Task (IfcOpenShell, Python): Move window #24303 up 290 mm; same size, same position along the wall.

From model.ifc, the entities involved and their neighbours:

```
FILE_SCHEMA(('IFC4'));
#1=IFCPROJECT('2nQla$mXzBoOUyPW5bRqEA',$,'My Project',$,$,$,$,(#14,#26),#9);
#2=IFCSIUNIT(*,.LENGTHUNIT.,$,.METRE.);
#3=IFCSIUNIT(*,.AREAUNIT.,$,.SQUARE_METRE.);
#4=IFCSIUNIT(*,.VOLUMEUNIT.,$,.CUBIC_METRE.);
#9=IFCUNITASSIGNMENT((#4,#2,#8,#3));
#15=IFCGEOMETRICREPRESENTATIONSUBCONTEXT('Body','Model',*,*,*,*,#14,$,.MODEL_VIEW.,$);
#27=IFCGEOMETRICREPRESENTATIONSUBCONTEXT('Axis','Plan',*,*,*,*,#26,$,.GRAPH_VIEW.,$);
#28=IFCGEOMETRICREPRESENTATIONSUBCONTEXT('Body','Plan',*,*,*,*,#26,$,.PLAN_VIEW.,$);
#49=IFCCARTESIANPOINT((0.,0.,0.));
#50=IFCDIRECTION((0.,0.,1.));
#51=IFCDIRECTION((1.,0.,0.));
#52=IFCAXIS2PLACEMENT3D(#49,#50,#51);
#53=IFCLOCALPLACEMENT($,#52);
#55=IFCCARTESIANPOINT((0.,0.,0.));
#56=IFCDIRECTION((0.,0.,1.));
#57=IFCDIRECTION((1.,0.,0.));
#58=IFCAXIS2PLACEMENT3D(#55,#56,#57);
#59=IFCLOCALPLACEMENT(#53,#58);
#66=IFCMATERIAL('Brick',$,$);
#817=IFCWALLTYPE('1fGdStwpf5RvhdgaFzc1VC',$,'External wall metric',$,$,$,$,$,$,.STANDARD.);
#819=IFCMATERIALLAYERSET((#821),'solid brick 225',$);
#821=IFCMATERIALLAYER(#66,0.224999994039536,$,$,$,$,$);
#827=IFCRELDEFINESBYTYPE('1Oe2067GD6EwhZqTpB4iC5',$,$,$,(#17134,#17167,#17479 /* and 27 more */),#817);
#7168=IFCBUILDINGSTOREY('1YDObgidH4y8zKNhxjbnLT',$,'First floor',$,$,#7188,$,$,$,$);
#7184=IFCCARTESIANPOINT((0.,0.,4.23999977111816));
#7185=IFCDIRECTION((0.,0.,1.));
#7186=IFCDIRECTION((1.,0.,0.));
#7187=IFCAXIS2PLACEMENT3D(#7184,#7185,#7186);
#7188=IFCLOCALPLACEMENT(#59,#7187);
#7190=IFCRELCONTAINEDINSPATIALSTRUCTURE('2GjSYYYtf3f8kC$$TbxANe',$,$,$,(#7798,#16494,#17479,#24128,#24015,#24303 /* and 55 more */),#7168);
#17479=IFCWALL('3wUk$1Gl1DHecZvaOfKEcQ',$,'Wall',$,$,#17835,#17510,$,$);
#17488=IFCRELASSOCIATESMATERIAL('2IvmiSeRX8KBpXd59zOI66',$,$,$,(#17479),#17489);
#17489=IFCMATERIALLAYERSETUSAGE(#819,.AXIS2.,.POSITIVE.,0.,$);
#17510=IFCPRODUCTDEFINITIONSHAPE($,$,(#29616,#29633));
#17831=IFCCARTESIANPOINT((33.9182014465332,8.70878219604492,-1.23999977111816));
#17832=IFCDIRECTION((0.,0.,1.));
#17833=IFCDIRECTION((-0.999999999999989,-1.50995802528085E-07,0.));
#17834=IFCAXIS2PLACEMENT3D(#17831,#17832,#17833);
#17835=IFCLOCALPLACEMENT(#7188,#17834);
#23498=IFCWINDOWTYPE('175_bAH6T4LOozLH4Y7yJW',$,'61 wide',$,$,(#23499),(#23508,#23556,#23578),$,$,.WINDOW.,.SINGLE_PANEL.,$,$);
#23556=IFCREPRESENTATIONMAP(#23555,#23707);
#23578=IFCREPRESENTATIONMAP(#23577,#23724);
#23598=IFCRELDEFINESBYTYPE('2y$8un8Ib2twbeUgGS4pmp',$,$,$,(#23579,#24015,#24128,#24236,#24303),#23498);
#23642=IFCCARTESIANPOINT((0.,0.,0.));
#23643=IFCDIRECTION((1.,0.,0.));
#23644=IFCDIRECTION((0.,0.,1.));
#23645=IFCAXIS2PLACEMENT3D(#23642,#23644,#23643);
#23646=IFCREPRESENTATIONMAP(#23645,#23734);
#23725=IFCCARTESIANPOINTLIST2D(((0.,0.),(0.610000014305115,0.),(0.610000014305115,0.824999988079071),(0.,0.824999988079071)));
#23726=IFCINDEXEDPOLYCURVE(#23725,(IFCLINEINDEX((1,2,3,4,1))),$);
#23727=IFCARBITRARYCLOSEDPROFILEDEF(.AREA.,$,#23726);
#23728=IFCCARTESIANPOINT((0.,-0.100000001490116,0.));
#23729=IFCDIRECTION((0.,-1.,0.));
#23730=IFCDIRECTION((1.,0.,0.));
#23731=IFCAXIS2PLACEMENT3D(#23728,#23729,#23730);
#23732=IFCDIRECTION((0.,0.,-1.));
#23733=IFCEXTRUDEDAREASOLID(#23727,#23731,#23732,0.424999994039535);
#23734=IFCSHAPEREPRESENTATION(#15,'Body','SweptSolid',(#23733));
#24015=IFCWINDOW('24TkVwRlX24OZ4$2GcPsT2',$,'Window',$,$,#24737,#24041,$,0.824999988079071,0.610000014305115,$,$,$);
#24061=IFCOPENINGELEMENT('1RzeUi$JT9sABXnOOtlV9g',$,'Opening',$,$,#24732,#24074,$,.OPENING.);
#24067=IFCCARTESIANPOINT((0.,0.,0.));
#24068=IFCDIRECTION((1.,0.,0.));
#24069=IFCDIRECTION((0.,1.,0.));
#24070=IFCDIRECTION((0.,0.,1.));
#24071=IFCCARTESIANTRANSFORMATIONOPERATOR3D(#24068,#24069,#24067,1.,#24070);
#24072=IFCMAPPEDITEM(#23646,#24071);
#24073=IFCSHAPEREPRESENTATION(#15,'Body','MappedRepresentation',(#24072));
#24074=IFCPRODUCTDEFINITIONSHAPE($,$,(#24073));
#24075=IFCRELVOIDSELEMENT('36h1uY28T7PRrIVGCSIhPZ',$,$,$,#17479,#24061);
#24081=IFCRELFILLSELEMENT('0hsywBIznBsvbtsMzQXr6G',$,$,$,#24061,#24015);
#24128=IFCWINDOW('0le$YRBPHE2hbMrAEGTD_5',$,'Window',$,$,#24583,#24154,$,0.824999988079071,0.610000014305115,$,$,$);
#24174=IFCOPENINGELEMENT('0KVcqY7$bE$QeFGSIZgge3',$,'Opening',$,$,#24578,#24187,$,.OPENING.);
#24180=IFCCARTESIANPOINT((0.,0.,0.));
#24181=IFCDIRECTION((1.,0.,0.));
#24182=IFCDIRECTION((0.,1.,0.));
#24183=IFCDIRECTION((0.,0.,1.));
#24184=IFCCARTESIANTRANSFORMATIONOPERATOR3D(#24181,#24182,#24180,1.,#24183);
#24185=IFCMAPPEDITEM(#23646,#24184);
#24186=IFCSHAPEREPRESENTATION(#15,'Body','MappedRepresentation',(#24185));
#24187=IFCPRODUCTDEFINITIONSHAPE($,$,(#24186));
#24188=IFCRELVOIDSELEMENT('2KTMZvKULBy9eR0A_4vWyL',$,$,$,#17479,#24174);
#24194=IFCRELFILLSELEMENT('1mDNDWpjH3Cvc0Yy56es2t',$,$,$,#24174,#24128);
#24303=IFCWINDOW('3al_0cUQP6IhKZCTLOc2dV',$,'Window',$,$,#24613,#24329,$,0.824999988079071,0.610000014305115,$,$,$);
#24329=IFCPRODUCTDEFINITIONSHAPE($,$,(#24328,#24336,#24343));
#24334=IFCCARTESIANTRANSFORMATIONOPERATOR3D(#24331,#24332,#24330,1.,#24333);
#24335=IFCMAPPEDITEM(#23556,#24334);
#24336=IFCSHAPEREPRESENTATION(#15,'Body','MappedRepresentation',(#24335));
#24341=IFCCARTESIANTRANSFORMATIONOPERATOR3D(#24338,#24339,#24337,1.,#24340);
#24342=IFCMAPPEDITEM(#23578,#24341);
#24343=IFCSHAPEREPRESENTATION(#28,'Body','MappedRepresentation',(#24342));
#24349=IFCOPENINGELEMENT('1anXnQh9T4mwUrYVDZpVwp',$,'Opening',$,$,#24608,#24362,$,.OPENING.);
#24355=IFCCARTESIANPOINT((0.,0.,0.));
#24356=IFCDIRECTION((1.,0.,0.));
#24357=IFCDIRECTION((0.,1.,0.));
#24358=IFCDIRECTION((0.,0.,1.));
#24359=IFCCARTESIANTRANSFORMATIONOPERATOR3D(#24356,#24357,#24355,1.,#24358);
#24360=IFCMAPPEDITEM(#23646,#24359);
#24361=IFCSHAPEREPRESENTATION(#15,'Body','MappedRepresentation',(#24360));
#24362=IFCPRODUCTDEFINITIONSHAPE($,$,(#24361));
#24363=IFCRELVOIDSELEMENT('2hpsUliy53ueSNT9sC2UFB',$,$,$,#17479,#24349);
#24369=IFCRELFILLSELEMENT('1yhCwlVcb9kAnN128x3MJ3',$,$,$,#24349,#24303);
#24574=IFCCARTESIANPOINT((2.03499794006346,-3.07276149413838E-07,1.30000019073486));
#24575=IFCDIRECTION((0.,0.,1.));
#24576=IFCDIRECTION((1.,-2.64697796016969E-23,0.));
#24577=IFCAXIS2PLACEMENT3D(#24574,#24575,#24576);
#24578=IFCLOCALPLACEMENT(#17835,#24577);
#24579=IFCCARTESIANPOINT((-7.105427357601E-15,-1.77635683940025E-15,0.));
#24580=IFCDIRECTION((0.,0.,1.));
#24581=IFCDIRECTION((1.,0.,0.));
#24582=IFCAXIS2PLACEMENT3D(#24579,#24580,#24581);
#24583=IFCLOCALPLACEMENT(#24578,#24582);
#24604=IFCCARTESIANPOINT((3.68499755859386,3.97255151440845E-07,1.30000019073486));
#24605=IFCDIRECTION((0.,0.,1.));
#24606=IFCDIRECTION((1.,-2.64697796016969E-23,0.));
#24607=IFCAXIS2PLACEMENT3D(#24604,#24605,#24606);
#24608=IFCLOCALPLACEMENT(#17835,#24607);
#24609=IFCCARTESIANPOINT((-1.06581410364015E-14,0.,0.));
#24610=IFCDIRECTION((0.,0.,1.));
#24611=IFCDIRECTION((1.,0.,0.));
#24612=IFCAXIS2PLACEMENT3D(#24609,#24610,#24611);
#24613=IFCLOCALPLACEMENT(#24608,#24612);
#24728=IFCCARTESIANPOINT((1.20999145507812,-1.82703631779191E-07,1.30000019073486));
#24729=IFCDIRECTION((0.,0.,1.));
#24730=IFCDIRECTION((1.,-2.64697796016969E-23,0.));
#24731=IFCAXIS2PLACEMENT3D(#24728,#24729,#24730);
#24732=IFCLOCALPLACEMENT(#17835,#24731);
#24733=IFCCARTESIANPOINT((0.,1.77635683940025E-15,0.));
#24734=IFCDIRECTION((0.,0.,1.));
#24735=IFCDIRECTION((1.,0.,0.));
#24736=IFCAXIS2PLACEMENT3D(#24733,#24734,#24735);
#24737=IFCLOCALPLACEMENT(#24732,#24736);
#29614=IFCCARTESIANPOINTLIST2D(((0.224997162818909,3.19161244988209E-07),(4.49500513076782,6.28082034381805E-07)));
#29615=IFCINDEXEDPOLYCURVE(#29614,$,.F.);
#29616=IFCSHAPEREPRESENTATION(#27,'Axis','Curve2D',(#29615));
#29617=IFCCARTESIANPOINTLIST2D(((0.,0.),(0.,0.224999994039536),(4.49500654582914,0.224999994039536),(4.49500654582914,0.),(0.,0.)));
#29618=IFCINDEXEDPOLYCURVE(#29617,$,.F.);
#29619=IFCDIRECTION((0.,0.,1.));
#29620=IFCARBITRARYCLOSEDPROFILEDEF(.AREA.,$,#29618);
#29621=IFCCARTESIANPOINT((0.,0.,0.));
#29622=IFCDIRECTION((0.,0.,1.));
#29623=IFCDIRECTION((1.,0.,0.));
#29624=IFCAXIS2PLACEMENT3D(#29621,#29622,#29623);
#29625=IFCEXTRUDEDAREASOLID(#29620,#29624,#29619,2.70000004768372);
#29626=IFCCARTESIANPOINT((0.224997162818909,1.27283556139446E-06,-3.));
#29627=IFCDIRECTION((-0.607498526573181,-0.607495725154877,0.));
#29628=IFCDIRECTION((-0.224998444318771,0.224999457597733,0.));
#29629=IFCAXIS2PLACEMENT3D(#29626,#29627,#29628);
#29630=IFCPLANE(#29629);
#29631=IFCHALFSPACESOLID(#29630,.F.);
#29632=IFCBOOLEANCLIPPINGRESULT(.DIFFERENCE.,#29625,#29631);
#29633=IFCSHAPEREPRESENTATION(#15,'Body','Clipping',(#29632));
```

```python
import numpy as np
import ifcopenshell
import ifcopenshell.api.geometry
import ifcopenshell.util.placement
import ifcopenshell.util.unit

model = ifcopenshell.open("model.ifc")
unit_scale = ifcopenshell.util.unit.calculate_unit_scale(model)

window = model.by_guid("3al_0cUQP6IhKZCTLOc2dV")
opening = window.FillsVoids[0].RelatingOpeningElement
dz = 0.29 / unit_scale

shift = np.array([0.0, 0.0, dz])
# The window is placed relative to its opening, so it follows when the opening moves.
matrix = ifcopenshell.util.placement.get_local_placement(opening.ObjectPlacement)
matrix[:3, 3] += shift
ifcopenshell.api.geometry.edit_object_placement(
    model, product=opening, matrix=matrix, is_si=False, should_transform_children=True
)

print(f"moved by {dz * unit_scale:+.3f} m")

model.write("model_updated.ifc")
```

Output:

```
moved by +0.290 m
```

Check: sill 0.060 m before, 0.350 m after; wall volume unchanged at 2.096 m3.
